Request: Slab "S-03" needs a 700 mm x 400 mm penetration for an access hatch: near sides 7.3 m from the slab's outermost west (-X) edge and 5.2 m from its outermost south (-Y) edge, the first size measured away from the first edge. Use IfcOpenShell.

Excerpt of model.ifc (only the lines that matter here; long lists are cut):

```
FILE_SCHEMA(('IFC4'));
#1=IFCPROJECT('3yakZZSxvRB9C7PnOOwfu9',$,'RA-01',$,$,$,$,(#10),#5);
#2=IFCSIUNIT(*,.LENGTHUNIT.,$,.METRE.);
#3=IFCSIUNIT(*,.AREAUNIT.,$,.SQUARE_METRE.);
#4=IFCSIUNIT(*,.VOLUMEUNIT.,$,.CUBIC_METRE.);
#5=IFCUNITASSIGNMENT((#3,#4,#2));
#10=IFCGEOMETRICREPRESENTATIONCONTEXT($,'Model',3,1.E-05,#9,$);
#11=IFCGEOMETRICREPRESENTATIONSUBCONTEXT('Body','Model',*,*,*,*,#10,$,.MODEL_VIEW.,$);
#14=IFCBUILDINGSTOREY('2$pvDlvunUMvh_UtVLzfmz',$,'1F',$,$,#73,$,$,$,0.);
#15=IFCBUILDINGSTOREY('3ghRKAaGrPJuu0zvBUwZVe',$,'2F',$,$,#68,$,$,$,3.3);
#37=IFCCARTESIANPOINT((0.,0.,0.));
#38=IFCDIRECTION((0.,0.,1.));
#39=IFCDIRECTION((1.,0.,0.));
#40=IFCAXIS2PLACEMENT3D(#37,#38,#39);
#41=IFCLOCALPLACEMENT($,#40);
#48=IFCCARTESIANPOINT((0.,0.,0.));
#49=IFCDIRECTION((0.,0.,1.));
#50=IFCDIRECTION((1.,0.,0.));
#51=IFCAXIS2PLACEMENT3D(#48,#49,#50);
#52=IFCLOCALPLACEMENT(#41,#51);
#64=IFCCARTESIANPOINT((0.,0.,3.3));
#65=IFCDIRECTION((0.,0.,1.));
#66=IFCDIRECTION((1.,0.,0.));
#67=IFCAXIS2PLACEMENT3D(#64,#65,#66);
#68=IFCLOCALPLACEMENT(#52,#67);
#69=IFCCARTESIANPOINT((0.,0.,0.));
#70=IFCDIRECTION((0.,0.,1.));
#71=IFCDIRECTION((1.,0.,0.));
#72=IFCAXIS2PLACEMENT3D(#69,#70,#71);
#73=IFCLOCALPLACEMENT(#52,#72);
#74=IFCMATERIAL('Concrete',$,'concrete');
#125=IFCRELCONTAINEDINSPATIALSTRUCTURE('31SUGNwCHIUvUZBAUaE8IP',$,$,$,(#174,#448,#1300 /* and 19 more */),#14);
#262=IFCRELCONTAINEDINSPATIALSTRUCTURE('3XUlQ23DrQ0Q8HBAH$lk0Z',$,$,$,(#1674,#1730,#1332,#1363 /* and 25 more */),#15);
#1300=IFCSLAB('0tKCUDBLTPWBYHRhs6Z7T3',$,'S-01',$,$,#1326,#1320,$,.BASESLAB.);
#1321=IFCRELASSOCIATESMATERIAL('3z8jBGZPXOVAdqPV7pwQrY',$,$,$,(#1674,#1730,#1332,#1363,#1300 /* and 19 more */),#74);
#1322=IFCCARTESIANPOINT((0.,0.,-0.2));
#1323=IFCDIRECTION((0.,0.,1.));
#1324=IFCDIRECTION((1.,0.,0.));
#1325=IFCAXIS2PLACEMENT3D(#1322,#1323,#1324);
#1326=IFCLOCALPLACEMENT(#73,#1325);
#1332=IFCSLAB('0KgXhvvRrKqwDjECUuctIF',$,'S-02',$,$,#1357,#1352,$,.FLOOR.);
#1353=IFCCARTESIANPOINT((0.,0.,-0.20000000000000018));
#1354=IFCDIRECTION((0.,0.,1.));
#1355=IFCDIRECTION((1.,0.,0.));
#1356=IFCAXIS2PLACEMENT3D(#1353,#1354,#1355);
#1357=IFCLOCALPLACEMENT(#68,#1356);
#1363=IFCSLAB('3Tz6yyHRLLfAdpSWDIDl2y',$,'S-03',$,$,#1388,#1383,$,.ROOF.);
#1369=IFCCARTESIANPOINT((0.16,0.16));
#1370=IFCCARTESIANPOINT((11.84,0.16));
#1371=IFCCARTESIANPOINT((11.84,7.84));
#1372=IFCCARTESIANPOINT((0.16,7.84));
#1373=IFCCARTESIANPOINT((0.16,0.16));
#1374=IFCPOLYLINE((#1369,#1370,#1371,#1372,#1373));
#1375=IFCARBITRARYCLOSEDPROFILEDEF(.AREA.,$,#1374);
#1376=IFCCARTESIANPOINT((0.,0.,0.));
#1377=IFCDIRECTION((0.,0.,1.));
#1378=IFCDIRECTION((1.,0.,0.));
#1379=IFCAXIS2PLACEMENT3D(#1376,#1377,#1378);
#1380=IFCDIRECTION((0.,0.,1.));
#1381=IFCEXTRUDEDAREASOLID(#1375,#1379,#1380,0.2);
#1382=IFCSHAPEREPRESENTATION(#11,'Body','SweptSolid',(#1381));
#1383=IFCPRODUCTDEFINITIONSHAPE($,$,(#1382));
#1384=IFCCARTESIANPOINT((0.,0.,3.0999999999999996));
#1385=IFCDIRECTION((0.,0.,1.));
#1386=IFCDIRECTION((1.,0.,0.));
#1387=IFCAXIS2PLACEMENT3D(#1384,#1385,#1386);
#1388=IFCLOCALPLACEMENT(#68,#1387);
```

```python
import numpy as np
import ifcopenshell
import ifcopenshell.api.feature
import ifcopenshell.api.geometry
import ifcopenshell.api.root
import ifcopenshell.geom
import ifcopenshell.util.placement
import ifcopenshell.util.representation
import ifcopenshell.util.shape
import ifcopenshell.util.unit

model = ifcopenshell.open("model.ifc")
unit_scale = ifcopenshell.util.unit.calculate_unit_scale(model)
settings = ifcopenshell.geom.settings()


def volume(element):
    """Net volume in cubic metres, openings subtracted."""
    shape = ifcopenshell.geom.create_shape(settings, element)
    return ifcopenshell.util.shape.get_volume(shape.geometry)


slab = model.by_guid("3Tz6yyHRLLfAdpSWDIDl2y")
before = volume(slab)

# Extent in the slab's own axes, in metres. The edges named are its -X and -Y sides.
slab_shape = ifcopenshell.geom.create_shape(settings, slab)
vertices = ifcopenshell.util.shape.get_vertices(slab_shape.geometry)
x_min, y_min, bottom = vertices.min(axis=0)
top = vertices[:, 2].max()

opening = ifcopenshell.api.root.create_entity(model, ifc_class="IfcOpeningElement", name="Access hatch opening", predefined_type="OPENING")
context = ifcopenshell.util.representation.get_context(model, "Model", "Body", "MODEL_VIEW")
width, depth = 0.7, 0.4
outline = [(0.0, 0.0), (width, 0.0), (width, depth), (0.0, depth), (0.0, 0.0)]
# Overshoot both faces by 50 mm so the cut is clean.
shape = ifcopenshell.api.geometry.add_slab_representation(
    model, context=context, depth=top - bottom + 0.1, polyline=outline
)
ifcopenshell.api.geometry.assign_representation(model, product=opening, representation=shape)

matrix = ifcopenshell.util.placement.get_local_placement(slab.ObjectPlacement)
matrix[:, 3] = matrix @ np.append(np.array([x_min + 7.3, y_min + 5.2, bottom - 0.05]) / unit_scale, 1.0)
ifcopenshell.api.geometry.edit_object_placement(model, product=opening, matrix=matrix, is_si=False)
ifcopenshell.api.feature.add_feature(model, feature=opening, element=slab)

after = volume(slab)

print(f"slab volume {before:.3f} -> {after:.3f} m3")

model.write("model_rev.ifc")
```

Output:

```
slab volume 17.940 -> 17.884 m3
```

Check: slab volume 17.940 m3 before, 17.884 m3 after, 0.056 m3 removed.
